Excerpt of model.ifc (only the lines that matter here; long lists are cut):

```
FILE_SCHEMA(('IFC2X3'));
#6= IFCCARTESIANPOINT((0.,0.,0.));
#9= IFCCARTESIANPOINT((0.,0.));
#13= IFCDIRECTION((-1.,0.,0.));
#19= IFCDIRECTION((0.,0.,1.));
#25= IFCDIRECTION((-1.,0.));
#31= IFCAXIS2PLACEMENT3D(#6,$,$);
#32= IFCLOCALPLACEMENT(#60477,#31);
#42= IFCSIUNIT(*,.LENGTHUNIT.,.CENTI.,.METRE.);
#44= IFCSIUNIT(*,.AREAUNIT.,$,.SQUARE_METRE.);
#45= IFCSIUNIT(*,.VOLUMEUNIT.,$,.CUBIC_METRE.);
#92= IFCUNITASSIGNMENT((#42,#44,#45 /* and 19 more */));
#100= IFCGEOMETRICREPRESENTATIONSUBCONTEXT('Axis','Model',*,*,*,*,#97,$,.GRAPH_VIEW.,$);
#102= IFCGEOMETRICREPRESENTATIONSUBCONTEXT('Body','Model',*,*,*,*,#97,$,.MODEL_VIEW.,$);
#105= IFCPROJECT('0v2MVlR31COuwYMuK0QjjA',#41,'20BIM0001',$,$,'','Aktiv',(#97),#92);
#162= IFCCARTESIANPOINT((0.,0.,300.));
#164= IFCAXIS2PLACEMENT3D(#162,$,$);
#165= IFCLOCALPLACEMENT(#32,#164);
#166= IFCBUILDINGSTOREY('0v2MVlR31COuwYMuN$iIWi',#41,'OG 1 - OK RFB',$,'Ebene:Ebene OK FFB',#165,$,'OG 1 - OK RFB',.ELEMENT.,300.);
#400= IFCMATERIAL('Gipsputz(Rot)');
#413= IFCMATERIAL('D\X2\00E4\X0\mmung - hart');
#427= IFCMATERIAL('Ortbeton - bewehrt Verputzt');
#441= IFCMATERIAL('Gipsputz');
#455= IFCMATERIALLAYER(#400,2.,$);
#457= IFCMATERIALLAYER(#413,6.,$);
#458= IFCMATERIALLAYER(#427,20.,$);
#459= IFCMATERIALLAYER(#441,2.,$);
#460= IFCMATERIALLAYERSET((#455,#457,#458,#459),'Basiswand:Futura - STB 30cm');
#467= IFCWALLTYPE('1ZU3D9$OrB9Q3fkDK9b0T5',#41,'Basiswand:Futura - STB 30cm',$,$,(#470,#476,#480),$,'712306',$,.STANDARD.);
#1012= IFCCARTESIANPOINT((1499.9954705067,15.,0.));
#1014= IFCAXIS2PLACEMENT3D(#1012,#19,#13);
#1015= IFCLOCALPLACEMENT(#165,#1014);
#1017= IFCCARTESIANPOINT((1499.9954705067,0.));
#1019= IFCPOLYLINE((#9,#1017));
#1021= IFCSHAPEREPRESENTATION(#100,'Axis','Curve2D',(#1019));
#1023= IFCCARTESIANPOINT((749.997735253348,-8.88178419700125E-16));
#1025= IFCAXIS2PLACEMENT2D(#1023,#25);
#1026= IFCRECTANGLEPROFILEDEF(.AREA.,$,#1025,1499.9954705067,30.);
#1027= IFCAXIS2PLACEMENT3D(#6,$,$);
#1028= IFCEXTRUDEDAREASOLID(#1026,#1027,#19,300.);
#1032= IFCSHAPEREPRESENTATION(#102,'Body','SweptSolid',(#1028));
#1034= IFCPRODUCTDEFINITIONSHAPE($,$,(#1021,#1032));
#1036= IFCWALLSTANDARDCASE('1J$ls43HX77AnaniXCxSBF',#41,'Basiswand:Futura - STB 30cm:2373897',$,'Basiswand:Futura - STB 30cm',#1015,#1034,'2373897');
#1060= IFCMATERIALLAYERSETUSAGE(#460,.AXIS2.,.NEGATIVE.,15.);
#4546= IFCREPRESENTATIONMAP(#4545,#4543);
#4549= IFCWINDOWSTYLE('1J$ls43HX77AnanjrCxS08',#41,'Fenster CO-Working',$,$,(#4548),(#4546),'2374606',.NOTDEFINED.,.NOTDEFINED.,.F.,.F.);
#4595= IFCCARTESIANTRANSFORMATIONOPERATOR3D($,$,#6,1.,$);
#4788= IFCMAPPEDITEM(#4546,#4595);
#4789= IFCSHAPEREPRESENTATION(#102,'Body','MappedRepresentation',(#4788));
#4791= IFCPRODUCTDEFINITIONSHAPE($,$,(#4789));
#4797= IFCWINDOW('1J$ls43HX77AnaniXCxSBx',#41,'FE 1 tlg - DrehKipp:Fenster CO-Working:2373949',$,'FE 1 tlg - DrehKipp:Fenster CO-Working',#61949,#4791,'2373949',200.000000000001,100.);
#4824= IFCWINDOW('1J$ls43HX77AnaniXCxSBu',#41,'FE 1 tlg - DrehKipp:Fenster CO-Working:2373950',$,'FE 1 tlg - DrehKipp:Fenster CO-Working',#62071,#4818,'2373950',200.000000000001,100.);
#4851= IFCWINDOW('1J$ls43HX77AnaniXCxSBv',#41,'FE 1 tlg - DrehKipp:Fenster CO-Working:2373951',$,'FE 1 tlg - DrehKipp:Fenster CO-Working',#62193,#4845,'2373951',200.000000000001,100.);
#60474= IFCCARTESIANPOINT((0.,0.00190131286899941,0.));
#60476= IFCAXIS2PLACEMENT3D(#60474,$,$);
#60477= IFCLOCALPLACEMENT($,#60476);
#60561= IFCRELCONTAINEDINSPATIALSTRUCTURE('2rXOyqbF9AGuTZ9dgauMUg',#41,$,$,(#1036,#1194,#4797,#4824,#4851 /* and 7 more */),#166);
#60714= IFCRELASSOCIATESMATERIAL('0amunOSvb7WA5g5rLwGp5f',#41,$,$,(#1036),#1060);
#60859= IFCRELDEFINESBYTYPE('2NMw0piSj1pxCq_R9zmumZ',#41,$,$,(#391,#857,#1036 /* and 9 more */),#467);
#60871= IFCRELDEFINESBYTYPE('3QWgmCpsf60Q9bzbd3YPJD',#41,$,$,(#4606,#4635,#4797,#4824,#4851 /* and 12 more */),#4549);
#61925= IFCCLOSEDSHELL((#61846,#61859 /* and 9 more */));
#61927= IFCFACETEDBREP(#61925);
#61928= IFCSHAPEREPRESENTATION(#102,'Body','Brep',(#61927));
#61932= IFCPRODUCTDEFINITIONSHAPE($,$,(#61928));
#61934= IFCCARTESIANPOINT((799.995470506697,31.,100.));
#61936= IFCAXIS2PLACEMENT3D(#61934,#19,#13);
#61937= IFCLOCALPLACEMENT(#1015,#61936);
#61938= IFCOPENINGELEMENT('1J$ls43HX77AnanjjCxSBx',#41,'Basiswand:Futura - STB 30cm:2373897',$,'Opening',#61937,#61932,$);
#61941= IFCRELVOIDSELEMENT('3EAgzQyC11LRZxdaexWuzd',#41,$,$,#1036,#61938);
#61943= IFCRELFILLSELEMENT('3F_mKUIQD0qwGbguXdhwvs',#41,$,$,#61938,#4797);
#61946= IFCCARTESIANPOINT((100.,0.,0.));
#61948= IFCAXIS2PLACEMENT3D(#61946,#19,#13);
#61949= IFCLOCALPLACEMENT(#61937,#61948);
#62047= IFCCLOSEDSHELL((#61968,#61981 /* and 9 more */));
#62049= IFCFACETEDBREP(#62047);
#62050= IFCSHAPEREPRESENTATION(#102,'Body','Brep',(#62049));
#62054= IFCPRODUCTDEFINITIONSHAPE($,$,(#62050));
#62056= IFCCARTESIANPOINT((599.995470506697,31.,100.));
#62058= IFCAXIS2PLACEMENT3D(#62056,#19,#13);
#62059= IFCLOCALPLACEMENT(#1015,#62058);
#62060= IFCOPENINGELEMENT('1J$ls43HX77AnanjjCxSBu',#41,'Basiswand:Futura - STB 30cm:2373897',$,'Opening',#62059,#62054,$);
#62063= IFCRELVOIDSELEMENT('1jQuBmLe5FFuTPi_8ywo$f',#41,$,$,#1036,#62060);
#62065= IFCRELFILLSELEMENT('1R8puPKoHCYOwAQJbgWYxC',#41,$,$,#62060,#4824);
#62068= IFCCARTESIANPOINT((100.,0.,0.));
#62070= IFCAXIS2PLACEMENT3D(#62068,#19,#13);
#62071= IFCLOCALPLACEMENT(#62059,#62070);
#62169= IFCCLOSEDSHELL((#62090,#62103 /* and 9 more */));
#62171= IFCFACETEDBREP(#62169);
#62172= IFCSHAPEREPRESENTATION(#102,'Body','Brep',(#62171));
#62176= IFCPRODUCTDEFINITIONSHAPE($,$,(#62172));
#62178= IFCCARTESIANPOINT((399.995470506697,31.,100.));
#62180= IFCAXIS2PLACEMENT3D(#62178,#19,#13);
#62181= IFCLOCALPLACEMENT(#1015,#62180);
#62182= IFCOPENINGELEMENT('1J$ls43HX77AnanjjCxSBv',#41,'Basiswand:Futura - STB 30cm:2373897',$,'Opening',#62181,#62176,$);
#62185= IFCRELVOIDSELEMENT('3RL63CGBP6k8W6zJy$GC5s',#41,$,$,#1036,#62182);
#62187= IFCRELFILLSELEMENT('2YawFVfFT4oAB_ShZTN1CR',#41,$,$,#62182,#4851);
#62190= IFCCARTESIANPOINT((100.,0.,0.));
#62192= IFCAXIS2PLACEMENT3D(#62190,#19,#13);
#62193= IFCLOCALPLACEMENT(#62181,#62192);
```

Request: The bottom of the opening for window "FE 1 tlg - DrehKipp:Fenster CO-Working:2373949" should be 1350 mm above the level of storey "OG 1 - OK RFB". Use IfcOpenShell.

```python
import numpy as np
import ifcopenshell
import ifcopenshell.api.geometry
import ifcopenshell.geom
import ifcopenshell.util.element
import ifcopenshell.util.placement
import ifcopenshell.util.shape
import ifcopenshell.util.unit

model = ifcopenshell.open("model.ifc")
unit_scale = ifcopenshell.util.unit.calculate_unit_scale(model)

window = model.by_guid("1J$ls43HX77AnaniXCxSBx")
opening = window.FillsVoids[0].RelatingOpeningElement
storey = ifcopenshell.util.element.get_container(window, ifc_class="IfcBuildingStorey")
level = ifcopenshell.util.placement.get_local_placement(storey.ObjectPlacement)[2, 3]

# The opening's origin need not be at the sill, so measure its lowest point.
shape = ifcopenshell.geom.create_shape(ifcopenshell.geom.settings(), opening)
bottom = ifcopenshell.util.shape.get_shape_bottom_elevation(shape, shape.geometry) / unit_scale
dz = level + 1.35 / unit_scale - bottom

shift = np.array([0.0, 0.0, dz])
# The window is placed relative to its opening, so it follows when the opening moves.
matrix = ifcopenshell.util.placement.get_local_placement(opening.ObjectPlacement)
matrix[:3, 3] += shift
ifcopenshell.api.geometry.edit_object_placement(
    model, product=opening, matrix=matrix, is_si=False, should_transform_children=True
)

print(f"moved by {dz * unit_scale:+.3f} m")

model.write("model_rev.ifc")
```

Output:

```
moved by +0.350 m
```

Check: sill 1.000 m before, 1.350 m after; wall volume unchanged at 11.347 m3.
